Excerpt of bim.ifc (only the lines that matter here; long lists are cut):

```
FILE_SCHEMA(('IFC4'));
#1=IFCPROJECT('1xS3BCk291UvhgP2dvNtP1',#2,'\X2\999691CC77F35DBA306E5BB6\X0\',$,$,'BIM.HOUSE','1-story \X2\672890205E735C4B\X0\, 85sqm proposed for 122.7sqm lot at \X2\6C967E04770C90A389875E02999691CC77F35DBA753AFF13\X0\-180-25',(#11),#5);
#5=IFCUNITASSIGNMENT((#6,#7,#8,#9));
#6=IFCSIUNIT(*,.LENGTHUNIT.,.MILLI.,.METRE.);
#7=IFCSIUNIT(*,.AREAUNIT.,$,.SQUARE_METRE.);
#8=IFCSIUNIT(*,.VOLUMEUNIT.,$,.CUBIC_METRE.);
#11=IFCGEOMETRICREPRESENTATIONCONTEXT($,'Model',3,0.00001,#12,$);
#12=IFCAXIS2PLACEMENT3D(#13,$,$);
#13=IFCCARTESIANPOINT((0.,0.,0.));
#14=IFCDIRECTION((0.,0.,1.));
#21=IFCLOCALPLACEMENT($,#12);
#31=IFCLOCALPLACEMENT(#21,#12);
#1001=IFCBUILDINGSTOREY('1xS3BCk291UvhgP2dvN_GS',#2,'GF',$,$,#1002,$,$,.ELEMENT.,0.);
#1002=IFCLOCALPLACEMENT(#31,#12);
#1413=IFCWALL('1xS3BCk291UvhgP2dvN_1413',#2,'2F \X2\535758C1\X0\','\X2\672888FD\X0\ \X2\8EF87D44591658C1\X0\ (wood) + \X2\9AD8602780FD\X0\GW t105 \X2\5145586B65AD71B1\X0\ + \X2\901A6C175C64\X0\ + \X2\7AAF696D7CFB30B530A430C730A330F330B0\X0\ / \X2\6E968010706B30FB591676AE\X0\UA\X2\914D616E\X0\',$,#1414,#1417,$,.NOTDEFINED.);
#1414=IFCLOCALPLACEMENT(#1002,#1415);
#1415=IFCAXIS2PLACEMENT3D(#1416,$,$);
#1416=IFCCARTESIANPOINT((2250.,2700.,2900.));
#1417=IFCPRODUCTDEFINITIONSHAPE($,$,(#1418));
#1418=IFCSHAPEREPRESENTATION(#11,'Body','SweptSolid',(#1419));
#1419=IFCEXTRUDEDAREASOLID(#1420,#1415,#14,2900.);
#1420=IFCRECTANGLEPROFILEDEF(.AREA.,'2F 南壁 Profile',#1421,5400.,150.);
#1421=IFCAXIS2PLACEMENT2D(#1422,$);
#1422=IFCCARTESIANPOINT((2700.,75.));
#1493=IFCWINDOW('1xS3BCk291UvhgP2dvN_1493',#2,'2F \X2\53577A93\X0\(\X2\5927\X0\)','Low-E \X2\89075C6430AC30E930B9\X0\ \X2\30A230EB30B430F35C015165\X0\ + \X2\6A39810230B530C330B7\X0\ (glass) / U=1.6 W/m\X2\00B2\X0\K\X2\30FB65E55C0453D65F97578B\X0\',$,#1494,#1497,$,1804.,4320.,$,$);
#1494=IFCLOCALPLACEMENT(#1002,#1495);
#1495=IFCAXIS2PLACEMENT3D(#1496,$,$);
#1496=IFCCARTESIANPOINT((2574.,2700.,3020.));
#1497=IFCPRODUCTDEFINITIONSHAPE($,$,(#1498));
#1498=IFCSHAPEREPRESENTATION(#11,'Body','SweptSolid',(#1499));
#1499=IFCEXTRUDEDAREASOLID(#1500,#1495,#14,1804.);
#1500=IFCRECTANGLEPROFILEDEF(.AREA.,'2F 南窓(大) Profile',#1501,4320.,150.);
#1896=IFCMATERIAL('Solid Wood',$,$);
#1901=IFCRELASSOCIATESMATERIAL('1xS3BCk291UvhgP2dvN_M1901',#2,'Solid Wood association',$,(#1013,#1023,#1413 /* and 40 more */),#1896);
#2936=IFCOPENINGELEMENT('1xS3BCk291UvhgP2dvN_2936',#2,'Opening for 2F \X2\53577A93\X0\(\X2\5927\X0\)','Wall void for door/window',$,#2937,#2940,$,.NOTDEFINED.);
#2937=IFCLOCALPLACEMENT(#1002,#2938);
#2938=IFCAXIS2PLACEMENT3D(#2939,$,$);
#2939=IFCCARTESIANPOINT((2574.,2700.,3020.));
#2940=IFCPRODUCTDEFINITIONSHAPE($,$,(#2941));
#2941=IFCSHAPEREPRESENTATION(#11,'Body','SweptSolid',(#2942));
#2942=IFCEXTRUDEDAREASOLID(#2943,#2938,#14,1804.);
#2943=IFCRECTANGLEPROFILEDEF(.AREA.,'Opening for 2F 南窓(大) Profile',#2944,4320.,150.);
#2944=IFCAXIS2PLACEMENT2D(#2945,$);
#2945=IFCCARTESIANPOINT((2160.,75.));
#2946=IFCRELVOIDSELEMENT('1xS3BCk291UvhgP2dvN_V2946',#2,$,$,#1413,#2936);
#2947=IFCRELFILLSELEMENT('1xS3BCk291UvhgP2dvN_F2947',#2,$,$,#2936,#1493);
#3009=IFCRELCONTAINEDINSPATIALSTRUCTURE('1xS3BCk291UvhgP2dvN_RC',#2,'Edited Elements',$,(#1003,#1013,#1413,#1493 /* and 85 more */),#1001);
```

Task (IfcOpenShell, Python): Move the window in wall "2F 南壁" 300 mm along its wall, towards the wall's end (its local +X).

```python
import ifcopenshell
import ifcopenshell.api.geometry
import ifcopenshell.util.placement
import ifcopenshell.util.unit

model = ifcopenshell.open("bim.ifc")
unit_scale = ifcopenshell.util.unit.calculate_unit_scale(model)

window = model.by_id(1493)
opening = window.FillsVoids[0].RelatingOpeningElement
wall = opening.VoidsElements[0].RelatingBuildingElement

wall_matrix = ifcopenshell.util.placement.get_local_placement(wall.ObjectPlacement)
shift = wall_matrix[:3, 0] * 0.3 / unit_scale
before = ifcopenshell.util.placement.get_local_placement(window.ObjectPlacement)[:3, 3].copy()

# The window is not placed relative to its opening, so move both.
for product in (opening, window):
    matrix = ifcopenshell.util.placement.get_local_placement(product.ObjectPlacement)
    matrix[:3, 3] += shift
    ifcopenshell.api.geometry.edit_object_placement(model, product=product, matrix=matrix, is_si=False)

after = ifcopenshell.util.placement.get_local_placement(window.ObjectPlacement)[:3, 3]
print("window moved by", (after - before).round(3) + 0.0)

model.write("bim_v2.ifc")
```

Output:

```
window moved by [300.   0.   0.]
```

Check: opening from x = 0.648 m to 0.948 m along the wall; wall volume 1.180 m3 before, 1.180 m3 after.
